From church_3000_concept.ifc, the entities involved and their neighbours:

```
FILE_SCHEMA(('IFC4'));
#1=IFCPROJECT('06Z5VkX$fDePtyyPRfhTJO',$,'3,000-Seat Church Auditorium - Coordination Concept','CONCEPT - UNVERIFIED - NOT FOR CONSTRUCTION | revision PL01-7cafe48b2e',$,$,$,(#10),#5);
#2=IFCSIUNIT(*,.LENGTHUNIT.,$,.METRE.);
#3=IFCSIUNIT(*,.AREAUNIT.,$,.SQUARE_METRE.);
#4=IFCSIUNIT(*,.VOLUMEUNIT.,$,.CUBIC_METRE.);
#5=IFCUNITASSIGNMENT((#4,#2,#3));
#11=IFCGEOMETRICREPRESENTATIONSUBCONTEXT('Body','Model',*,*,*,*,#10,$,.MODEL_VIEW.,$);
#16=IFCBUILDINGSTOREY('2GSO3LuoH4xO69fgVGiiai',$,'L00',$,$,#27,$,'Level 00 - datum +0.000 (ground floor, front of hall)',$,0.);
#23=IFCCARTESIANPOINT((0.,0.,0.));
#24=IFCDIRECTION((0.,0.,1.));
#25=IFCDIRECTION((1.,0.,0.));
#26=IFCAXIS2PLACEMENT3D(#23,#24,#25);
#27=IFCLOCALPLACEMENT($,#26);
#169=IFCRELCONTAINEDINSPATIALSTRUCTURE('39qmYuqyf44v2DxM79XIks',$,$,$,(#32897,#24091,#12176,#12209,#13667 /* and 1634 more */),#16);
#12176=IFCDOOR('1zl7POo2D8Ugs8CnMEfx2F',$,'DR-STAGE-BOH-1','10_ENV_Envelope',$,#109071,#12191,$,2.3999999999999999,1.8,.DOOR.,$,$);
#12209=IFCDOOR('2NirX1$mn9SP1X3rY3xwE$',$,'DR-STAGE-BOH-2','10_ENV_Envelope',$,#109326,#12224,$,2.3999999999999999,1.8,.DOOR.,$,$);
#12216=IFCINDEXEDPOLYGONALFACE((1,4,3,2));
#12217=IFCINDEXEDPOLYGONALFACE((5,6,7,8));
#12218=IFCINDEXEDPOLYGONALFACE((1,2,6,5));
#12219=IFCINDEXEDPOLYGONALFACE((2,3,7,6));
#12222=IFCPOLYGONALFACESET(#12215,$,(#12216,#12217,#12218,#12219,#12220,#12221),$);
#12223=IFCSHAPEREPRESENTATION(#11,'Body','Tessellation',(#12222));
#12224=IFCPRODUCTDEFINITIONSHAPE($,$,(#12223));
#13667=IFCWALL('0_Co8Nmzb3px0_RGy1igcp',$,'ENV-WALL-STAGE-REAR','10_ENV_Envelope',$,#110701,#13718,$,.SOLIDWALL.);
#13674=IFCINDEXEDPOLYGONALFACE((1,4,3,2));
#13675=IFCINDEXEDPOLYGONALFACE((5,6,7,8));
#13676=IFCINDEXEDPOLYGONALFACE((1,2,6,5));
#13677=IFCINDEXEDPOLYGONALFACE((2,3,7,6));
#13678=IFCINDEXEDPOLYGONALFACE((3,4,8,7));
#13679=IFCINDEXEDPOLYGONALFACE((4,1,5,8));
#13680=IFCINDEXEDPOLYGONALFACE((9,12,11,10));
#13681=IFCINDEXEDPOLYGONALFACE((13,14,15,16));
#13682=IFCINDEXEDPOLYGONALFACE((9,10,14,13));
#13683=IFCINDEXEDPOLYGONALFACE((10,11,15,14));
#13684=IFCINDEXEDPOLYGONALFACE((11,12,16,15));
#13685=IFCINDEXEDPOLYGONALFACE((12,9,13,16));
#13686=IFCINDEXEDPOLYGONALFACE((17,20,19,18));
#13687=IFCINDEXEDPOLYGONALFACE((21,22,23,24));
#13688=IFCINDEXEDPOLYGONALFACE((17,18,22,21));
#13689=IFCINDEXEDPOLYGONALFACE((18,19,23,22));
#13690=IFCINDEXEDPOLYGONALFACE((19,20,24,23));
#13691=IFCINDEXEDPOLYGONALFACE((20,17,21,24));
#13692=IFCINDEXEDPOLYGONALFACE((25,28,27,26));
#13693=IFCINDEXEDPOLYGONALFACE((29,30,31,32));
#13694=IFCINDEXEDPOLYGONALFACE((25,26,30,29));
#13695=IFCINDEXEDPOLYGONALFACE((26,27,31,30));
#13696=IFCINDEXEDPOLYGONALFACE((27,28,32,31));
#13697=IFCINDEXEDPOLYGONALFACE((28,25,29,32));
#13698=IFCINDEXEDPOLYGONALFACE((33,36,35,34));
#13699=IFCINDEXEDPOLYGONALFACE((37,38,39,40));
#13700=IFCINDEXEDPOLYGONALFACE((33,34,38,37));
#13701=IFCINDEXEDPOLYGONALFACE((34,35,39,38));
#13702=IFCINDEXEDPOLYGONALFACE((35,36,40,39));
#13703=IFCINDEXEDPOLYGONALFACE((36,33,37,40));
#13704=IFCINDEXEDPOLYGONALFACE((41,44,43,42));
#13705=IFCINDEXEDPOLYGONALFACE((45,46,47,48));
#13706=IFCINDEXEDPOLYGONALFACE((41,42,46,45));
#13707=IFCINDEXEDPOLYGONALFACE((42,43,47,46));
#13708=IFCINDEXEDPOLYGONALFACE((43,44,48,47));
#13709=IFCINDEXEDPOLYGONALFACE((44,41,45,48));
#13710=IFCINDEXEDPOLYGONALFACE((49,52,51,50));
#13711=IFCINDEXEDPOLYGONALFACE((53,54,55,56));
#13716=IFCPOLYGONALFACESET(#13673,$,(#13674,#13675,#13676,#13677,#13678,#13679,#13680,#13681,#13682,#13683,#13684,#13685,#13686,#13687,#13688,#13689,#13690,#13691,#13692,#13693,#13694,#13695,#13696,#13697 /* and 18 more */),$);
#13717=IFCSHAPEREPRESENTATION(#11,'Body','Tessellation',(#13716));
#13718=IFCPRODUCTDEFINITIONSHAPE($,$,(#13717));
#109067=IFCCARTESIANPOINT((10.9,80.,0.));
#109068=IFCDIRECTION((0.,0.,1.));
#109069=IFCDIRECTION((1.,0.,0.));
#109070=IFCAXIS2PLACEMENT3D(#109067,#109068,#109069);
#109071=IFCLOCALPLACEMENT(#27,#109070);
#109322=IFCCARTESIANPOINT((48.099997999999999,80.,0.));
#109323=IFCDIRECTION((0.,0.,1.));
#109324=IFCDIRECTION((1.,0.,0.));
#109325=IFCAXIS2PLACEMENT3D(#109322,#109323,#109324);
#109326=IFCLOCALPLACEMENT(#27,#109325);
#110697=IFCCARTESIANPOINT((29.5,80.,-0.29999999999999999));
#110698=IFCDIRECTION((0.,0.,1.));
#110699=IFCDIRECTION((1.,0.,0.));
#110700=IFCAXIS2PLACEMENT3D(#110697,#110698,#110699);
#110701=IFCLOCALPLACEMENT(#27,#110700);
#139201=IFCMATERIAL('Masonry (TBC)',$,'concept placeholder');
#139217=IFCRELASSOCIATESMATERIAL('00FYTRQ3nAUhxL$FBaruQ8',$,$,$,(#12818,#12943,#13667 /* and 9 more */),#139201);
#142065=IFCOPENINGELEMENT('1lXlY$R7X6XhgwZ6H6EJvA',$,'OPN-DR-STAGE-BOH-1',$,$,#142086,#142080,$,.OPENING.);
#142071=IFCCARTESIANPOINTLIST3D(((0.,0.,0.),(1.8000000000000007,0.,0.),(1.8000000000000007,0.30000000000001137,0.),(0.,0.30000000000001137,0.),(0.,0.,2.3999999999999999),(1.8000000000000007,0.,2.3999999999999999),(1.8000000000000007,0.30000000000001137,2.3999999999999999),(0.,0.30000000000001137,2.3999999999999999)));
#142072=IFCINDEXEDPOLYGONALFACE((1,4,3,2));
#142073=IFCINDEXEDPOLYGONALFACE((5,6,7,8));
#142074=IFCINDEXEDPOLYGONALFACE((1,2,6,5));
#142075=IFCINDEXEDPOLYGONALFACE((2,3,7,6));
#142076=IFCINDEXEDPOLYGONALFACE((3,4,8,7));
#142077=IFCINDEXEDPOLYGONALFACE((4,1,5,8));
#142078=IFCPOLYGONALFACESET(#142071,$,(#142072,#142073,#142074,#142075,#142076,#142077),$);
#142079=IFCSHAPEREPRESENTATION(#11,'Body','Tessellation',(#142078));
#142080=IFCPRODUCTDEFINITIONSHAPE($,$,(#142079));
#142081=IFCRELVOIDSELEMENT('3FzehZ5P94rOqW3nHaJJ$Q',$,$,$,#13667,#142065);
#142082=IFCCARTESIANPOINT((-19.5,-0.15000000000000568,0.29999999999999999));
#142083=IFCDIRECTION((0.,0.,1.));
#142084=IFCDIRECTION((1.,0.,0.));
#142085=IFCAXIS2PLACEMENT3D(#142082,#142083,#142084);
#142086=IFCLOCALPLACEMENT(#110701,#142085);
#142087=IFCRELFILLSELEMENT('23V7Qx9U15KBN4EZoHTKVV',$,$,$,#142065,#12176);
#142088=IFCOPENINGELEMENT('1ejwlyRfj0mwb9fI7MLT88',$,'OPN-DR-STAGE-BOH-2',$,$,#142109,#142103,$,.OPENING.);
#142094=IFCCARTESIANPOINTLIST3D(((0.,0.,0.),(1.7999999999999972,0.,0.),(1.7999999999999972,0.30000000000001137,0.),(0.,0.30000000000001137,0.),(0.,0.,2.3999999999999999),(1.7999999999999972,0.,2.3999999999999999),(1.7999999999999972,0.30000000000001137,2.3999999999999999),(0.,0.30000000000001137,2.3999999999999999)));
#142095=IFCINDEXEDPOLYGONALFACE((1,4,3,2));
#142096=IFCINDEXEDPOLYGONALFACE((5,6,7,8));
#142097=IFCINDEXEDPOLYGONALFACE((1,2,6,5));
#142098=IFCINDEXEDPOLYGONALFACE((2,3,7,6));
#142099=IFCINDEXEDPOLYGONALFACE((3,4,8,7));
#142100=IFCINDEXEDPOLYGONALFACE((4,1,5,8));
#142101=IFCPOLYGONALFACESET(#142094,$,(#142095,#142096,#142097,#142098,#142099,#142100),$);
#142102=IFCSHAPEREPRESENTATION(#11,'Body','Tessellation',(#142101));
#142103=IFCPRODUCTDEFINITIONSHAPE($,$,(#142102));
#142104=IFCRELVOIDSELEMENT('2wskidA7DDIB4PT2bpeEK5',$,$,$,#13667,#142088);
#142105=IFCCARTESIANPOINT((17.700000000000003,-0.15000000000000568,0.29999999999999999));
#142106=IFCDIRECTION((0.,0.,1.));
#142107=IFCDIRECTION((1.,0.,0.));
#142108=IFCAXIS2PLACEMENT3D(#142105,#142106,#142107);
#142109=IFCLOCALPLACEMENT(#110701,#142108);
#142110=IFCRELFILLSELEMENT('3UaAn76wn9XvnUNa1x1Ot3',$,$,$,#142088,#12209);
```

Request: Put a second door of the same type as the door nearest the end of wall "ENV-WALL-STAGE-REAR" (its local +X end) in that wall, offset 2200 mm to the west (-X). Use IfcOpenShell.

```python
import ifcopenshell
import ifcopenshell.api.feature
import ifcopenshell.api.geometry
import ifcopenshell.api.root
import ifcopenshell.geom
import ifcopenshell.util.element
import ifcopenshell.util.placement
import ifcopenshell.util.shape
import ifcopenshell.util.unit

model = ifcopenshell.open("church_3000_concept.ifc")
unit_scale = ifcopenshell.util.unit.calculate_unit_scale(model)
settings = ifcopenshell.geom.settings()


def volume(element):
    """Net volume in cubic metres, openings subtracted."""
    shape = ifcopenshell.geom.create_shape(settings, element)
    return ifcopenshell.util.shape.get_volume(shape.geometry)


door = model.by_guid("2NirX1$mn9SP1X3rY3xwE$")
opening = door.FillsVoids[0].RelatingOpeningElement
wall = opening.VoidsElements[0].RelatingBuildingElement
before = volume(wall)
shift = ifcopenshell.util.placement.get_local_placement(wall.ObjectPlacement)[:3, 0] * -2.2 / unit_scale

# copy_class copies the void relationship, type, container and properties, but no geometry.
new_opening = ifcopenshell.api.root.copy_class(model, product=opening)
new_opening.Representation = ifcopenshell.util.element.copy_deep(
    model, opening.Representation, exclude=["IfcGeometricRepresentationContext", "IfcRepresentationMap"]
)
new_door = ifcopenshell.api.root.copy_class(model, product=door)
new_door.Representation = ifcopenshell.util.element.copy_deep(
    model, door.Representation, exclude=["IfcGeometricRepresentationContext", "IfcRepresentationMap"]
)
ifcopenshell.api.feature.add_filling(model, opening=new_opening, element=new_door)

for old, new in ((opening, new_opening), (door, new_door)):
    matrix = ifcopenshell.util.placement.get_local_placement(old.ObjectPlacement)
    matrix[:3, 3] += shift
    ifcopenshell.api.geometry.edit_object_placement(model, product=new, matrix=matrix, is_si=False)

after = volume(wall)

print(f"wall volume {before:.3f} -> {after:.3f} m3")

model.write("church_3000_concept_v2.ifc")
```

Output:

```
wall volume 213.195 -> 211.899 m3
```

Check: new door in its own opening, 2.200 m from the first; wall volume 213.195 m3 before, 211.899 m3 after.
